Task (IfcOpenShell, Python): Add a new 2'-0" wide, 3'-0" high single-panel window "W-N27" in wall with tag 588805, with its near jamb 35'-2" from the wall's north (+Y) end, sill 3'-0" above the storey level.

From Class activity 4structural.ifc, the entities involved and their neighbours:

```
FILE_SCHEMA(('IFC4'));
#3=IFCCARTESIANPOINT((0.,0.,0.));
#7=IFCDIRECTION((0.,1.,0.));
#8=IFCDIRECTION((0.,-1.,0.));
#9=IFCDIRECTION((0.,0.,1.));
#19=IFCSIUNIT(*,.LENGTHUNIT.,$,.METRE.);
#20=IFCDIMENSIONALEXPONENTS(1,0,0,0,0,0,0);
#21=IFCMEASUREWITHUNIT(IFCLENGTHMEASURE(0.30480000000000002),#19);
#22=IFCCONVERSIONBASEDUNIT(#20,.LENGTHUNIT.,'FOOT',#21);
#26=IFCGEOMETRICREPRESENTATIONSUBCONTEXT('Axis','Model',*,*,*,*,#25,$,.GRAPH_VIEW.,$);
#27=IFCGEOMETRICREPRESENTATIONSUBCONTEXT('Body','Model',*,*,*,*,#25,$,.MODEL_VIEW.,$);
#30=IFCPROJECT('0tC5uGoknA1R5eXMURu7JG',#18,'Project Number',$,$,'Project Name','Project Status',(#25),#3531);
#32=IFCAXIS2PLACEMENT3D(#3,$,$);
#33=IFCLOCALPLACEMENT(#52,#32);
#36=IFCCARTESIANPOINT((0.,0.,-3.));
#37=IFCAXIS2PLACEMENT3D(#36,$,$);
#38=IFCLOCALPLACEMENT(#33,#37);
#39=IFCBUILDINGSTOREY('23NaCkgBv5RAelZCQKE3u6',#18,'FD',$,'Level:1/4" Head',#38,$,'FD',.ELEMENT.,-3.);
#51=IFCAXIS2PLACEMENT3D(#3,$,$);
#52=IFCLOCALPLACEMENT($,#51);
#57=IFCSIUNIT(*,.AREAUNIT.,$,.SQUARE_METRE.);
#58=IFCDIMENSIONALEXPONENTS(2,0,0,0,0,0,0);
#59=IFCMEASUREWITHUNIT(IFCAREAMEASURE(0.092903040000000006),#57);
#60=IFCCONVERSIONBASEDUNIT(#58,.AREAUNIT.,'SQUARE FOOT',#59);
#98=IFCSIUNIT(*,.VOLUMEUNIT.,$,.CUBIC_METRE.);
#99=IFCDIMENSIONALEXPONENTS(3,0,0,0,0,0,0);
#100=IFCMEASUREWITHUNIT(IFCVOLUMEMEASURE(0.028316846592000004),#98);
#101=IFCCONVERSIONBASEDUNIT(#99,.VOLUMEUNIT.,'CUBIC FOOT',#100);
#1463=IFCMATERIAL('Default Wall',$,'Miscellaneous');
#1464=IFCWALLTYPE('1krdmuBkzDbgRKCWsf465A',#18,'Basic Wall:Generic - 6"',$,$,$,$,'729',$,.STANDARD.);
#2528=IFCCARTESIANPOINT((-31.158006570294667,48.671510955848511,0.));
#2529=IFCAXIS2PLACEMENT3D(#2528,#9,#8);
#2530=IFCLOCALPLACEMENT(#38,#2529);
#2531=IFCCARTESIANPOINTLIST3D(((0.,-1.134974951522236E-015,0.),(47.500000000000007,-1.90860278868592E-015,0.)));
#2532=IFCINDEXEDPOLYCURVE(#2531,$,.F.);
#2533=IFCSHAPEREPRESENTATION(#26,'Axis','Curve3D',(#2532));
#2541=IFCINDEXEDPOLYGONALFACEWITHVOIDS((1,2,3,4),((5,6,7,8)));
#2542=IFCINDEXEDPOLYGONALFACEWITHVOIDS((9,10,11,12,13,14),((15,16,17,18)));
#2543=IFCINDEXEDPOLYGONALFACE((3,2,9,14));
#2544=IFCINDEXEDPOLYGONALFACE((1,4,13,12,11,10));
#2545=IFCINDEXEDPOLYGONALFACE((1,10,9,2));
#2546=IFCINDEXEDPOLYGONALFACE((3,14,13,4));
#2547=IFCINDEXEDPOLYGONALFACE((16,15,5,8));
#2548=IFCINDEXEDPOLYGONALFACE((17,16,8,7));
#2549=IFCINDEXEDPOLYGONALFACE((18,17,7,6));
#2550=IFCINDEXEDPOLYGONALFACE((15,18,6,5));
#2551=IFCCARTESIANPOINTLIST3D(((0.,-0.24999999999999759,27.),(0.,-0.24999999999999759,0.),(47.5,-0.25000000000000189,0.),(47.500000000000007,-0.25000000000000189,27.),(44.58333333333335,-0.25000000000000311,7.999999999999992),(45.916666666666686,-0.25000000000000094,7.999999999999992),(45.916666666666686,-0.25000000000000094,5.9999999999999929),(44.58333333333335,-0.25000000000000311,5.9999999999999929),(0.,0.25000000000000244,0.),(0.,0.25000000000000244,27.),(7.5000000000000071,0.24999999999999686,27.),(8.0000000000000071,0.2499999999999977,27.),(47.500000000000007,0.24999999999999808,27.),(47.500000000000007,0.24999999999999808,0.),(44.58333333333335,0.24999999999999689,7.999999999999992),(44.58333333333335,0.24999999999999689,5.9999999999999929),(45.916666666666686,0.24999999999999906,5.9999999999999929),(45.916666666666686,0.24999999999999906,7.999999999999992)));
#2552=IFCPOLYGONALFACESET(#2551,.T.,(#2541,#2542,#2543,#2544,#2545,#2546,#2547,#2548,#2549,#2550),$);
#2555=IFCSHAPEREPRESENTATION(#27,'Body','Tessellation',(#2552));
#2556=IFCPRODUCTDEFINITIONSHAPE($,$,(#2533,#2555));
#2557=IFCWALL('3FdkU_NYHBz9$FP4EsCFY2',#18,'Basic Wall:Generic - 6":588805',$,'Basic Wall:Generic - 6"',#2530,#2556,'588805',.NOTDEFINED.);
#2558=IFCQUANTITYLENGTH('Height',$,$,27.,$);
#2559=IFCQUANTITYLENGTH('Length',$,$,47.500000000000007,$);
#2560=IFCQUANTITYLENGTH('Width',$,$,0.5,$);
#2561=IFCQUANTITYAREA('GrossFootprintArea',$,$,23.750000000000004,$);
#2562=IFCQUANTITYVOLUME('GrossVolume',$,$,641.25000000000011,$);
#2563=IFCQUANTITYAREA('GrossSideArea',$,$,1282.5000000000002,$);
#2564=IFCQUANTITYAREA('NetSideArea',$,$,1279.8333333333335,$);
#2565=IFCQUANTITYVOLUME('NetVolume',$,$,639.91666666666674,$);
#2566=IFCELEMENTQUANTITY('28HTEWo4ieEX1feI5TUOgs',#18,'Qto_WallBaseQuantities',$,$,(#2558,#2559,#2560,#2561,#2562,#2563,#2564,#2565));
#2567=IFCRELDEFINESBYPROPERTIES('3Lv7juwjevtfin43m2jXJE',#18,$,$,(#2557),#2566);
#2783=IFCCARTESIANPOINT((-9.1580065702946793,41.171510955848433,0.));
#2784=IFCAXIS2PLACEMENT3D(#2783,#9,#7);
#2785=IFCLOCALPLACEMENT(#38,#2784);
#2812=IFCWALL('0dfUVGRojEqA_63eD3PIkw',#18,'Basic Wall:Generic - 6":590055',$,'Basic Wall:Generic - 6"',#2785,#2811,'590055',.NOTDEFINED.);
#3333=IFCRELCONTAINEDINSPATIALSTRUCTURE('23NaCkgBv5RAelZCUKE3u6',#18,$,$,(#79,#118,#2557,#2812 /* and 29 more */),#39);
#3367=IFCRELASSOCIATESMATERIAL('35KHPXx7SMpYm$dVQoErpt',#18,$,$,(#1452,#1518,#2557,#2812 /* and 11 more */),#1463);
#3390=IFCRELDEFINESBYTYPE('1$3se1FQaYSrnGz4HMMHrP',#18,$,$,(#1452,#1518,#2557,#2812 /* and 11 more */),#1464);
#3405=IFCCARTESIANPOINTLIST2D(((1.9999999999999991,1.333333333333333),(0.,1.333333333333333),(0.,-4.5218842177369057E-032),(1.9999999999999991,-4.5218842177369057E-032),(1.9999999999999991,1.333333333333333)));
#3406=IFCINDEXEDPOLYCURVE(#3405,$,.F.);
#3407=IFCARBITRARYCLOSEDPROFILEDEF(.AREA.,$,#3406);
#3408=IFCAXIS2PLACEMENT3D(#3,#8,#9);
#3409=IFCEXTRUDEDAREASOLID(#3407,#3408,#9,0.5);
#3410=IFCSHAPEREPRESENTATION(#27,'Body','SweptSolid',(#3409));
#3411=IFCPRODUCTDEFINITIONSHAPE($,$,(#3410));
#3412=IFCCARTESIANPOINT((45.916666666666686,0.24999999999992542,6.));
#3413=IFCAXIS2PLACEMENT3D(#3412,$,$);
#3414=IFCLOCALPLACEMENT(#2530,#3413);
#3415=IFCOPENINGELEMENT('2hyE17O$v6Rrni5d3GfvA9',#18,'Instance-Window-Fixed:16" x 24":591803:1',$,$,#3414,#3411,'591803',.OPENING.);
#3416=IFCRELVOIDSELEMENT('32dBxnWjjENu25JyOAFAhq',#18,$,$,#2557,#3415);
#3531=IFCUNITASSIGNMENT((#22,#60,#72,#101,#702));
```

```python
import numpy as np
import ifcopenshell
import ifcopenshell.api.feature
import ifcopenshell.api.geometry
import ifcopenshell.api.pset
import ifcopenshell.api.root
import ifcopenshell.api.spatial
import ifcopenshell.geom
import ifcopenshell.util.element
import ifcopenshell.util.placement
import ifcopenshell.util.representation
import ifcopenshell.util.shape
import ifcopenshell.util.unit

model = ifcopenshell.open("Class activity 4structural.ifc")
unit_scale = ifcopenshell.util.unit.calculate_unit_scale(model)
area_scale = ifcopenshell.util.unit.calculate_unit_scale(model, "AREAUNIT")
volume_scale = ifcopenshell.util.unit.calculate_unit_scale(model, "VOLUMEUNIT")
settings = ifcopenshell.geom.settings()


def volume(element):
    """Net volume in cubic metres, openings subtracted."""
    shape = ifcopenshell.geom.create_shape(settings, element)
    return ifcopenshell.util.shape.get_volume(shape.geometry)


wall = model.by_id(2557)
storey = ifcopenshell.util.element.get_container(wall, ifc_class="IfcBuildingStorey")
context = ifcopenshell.util.representation.get_context(model, "Model", "Body", "MODEL_VIEW")
before = volume(wall)

width, height, from_end, sill = 0.6096, 0.9144, 10.7188, 0.9144  # metres

# The wall runs along its own X axis, and the end named is its -X end.
wall_shape = ifcopenshell.geom.create_shape(settings, wall)
x, y, z = ifcopenshell.util.shape.get_vertices(wall_shape.geometry).T
start = x.min() + from_end
face, thickness = float(y.min()), float(y.max() - y.min())
wall_matrix = ifcopenshell.util.placement.get_local_placement(wall.ObjectPlacement)
level = ifcopenshell.util.placement.get_local_placement(storey.ObjectPlacement)[2, 3]


def in_wall(x, y):
    """Placement at x, y metres in the wall's axes, at sill height."""
    matrix = wall_matrix.copy()
    matrix[:, 3] = wall_matrix @ np.array([x / unit_scale, y / unit_scale, 0.0, 1.0])
    matrix[2, 3] = level + sill / unit_scale
    return matrix


# Opening: a box that overshoots both wall faces by 50 mm.
opening = ifcopenshell.api.root.create_entity(model, ifc_class="IfcOpeningElement", predefined_type="OPENING")
box = ifcopenshell.api.geometry.add_wall_representation(
    model, context=context, length=width, height=height, thickness=thickness + 0.1
)
ifcopenshell.api.geometry.assign_representation(model, product=opening, representation=box)
ifcopenshell.api.geometry.edit_object_placement(model, product=opening, matrix=in_wall(start, face - 0.05), is_si=False)
ifcopenshell.api.feature.add_feature(model, feature=opening, element=wall)

window = ifcopenshell.api.root.create_entity(model, ifc_class="IfcWindow", name="W-N27", predefined_type="WINDOW")
window.OverallWidth, window.OverallHeight = width / unit_scale, height / unit_scale
window.PartitioningType = "SINGLE_PANEL"
body = ifcopenshell.api.geometry.add_window_representation(
    model,
    context=context,
    overall_width=window.OverallWidth,
    overall_height=window.OverallHeight,
    partition_type="SINGLE_PANEL",
)
ifcopenshell.api.geometry.assign_representation(model, product=window, representation=body)
ifcopenshell.api.spatial.assign_container(model, products=[window], relating_structure=storey)
ifcopenshell.api.feature.add_filling(model, opening=opening, element=window)

# Centre the window in the wall's thickness.
ifcopenshell.api.geometry.edit_object_placement(model, product=window, matrix=in_wall(start, face), is_si=False)
window_shape = ifcopenshell.geom.create_shape(settings, window)
depth = ifcopenshell.util.shape.get_vertices(window_shape.geometry)[:, 1]
offset = face + thickness / 2 - (depth.min() + depth.max()) / 2
ifcopenshell.api.geometry.edit_object_placement(model, product=window, matrix=in_wall(start, offset), is_si=False)

after = volume(wall)

# Update the wall's stored quantities.
qto = model.by_id(ifcopenshell.util.element.get_pset(wall, "Qto_WallBaseQuantities", should_inherit=False)["id"])
ifcopenshell.api.pset.edit_qto(model, qto=qto, properties={
    "NetSideArea": after / thickness / area_scale,
    "NetVolume": after / volume_scale,
})

print(f"wall volume {before:.3f} -> {after:.3f} m3")

model.write("Class activity 4structural_rev.ifc")
```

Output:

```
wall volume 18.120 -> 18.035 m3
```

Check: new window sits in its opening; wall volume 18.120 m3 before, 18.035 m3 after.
